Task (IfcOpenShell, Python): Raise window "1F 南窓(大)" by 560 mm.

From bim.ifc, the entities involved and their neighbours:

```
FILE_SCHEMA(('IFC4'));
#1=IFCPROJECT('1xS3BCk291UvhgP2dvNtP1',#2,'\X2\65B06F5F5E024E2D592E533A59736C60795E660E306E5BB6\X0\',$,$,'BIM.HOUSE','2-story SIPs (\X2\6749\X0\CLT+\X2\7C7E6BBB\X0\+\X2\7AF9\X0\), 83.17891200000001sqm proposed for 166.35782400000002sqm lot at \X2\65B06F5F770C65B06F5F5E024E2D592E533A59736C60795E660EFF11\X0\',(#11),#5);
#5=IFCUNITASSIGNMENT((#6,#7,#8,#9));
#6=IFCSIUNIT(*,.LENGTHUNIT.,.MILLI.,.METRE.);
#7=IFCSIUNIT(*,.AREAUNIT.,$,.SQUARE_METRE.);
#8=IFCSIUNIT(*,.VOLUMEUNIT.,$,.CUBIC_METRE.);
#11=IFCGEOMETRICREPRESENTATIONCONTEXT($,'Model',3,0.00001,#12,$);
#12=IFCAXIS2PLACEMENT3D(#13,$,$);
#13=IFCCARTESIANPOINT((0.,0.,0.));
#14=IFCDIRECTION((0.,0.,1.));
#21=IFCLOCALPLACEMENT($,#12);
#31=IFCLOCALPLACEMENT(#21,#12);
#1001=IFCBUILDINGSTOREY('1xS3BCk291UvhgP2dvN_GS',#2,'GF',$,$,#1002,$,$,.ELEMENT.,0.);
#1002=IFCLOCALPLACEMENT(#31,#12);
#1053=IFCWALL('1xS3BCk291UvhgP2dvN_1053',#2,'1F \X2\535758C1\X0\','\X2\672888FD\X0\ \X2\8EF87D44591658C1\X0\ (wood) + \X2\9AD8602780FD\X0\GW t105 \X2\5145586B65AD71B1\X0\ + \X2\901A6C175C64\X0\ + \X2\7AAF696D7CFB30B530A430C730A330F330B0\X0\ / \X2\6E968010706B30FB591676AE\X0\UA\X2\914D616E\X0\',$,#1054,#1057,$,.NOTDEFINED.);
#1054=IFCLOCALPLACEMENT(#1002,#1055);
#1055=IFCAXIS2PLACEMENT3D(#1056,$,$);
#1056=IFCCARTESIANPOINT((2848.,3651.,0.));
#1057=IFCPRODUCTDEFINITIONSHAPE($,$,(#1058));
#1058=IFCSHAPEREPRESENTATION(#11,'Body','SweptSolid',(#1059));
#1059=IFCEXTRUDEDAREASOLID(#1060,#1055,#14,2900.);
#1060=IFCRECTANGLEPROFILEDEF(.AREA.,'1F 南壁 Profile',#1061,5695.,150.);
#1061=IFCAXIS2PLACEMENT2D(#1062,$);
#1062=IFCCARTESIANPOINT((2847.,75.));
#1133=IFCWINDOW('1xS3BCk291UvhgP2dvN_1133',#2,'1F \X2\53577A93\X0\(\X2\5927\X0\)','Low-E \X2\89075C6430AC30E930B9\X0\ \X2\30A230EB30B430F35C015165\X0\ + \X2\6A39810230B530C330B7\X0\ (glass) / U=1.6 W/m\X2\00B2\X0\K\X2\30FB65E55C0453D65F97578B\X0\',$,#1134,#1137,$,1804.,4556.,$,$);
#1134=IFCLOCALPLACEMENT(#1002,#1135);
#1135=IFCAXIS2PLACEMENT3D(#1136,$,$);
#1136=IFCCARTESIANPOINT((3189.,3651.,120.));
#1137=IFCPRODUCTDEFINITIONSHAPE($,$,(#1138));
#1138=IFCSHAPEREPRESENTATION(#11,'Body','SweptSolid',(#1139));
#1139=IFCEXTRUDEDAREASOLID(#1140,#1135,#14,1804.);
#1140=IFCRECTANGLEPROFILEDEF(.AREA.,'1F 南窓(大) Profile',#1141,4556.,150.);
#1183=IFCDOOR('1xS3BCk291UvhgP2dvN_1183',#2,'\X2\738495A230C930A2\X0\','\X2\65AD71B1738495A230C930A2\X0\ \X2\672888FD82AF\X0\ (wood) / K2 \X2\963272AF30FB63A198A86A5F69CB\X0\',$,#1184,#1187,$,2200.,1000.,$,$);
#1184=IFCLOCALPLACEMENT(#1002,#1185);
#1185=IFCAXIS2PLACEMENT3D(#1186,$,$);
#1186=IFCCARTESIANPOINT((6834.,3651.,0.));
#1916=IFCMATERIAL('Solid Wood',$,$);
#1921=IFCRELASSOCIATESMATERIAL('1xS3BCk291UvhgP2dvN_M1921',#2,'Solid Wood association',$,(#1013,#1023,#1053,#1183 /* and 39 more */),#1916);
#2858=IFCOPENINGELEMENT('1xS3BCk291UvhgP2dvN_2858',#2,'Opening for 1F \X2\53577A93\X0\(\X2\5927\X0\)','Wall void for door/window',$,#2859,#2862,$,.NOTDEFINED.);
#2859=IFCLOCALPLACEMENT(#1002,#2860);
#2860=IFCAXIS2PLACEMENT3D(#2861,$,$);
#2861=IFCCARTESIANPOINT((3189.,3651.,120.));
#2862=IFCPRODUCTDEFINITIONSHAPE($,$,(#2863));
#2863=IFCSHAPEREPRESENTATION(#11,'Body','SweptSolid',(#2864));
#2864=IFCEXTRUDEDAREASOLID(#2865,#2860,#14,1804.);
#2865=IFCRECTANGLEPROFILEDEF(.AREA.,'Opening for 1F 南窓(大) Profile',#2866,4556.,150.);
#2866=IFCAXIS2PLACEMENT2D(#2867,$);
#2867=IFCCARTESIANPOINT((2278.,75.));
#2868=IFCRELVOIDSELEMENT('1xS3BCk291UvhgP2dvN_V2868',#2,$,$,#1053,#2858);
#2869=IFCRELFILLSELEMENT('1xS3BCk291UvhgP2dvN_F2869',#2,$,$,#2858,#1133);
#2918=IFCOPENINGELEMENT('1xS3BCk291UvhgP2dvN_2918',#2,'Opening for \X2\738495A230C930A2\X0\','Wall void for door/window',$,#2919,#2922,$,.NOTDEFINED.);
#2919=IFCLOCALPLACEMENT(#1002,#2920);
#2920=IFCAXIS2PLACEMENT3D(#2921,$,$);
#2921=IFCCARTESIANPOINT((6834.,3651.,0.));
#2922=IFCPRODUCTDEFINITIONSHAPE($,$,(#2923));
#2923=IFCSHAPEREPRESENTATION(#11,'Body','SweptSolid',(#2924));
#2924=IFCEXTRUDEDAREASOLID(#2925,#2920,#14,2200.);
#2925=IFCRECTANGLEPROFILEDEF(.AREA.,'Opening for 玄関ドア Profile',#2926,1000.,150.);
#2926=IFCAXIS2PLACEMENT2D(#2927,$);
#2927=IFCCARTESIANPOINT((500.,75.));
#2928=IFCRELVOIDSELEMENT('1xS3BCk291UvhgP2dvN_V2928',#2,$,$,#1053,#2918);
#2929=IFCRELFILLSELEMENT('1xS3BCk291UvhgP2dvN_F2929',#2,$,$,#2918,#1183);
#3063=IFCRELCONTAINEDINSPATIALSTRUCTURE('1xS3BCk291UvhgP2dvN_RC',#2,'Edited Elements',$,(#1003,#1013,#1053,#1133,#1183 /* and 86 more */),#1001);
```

```python
import numpy as np
import ifcopenshell
import ifcopenshell.api.geometry
import ifcopenshell.util.placement
import ifcopenshell.util.unit

model = ifcopenshell.open("bim.ifc")
unit_scale = ifcopenshell.util.unit.calculate_unit_scale(model)

window = model.by_guid("1xS3BCk291UvhgP2dvN_1133")
opening = window.FillsVoids[0].RelatingOpeningElement
dz = 560.0

shift = np.array([0.0, 0.0, dz])
# The window is not placed relative to its opening, so move both.
for product in (opening, window):
    matrix = ifcopenshell.util.placement.get_local_placement(product.ObjectPlacement)
    matrix[:3, 3] += shift
    ifcopenshell.api.geometry.edit_object_placement(model, product=product, matrix=matrix, is_si=False)

print(f"moved by {dz * unit_scale:+.3f} m")

model.write("bim_v2.ifc")
```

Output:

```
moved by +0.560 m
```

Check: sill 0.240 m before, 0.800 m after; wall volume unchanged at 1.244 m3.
